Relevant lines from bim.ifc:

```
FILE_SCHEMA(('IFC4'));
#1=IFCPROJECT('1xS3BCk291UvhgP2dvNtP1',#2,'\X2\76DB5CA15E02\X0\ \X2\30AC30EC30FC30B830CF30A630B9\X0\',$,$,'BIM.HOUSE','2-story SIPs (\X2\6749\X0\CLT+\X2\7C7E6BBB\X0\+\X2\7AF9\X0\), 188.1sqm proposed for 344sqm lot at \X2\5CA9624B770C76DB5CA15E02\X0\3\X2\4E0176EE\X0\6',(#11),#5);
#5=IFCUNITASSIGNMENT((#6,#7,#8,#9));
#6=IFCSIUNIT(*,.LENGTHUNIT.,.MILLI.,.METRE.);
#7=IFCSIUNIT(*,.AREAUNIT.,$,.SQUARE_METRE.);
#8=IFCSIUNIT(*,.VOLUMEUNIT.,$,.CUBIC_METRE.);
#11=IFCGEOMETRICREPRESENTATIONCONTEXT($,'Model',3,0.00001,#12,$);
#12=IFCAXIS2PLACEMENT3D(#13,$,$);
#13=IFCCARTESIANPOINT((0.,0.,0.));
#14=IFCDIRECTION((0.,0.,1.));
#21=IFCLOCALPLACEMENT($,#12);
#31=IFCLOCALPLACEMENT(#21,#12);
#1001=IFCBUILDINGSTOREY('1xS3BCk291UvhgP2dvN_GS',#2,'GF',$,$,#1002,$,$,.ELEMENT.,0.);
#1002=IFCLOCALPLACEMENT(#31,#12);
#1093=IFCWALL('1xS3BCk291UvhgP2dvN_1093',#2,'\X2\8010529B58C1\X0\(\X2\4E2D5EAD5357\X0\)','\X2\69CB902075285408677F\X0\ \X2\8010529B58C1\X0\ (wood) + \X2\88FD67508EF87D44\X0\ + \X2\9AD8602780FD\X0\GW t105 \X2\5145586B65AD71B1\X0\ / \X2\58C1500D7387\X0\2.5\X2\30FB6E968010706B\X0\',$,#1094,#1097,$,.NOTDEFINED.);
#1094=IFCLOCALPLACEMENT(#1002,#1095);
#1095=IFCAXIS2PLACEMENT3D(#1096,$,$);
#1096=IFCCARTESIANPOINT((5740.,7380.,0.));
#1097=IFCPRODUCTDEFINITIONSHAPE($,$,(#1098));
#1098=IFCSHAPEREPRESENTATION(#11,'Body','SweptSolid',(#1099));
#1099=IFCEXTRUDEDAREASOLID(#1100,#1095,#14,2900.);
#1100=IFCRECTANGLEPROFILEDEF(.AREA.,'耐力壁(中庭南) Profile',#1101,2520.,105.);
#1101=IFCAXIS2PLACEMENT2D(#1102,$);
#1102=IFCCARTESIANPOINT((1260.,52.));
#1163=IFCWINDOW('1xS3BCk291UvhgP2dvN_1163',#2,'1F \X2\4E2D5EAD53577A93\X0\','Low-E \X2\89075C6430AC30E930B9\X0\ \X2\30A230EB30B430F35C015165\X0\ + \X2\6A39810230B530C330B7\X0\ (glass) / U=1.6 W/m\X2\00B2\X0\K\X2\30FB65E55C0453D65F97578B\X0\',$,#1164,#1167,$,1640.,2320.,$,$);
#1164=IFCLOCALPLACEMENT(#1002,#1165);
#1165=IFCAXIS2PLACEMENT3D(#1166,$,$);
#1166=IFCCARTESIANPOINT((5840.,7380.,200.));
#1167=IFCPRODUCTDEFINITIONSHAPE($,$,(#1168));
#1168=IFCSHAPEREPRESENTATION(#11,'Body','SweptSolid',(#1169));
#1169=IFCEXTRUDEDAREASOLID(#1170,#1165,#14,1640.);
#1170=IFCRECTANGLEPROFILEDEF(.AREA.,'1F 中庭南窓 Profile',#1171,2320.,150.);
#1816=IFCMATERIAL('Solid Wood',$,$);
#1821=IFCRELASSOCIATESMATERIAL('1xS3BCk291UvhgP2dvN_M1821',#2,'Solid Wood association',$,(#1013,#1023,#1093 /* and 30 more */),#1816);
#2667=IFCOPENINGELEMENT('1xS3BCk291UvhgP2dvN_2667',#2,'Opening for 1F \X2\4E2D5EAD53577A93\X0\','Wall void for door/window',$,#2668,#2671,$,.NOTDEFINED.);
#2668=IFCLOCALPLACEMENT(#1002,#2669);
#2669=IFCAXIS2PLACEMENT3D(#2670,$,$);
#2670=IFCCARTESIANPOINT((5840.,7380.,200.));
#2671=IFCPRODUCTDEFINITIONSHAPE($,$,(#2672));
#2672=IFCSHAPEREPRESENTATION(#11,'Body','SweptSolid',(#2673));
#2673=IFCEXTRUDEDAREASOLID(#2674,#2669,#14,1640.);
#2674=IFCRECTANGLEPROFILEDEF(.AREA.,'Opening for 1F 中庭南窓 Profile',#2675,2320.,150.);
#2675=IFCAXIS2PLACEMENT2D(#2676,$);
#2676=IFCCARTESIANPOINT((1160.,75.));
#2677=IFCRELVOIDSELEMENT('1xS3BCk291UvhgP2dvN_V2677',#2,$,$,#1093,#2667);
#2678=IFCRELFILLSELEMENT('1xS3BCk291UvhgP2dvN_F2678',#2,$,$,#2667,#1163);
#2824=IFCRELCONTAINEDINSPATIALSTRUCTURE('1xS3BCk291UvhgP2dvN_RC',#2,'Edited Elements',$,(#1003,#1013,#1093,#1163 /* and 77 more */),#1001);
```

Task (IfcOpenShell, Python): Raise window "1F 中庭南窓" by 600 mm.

```python
import numpy as np
import ifcopenshell
import ifcopenshell.api.geometry
import ifcopenshell.util.placement
import ifcopenshell.util.unit

model = ifcopenshell.open("bim.ifc")
unit_scale = ifcopenshell.util.unit.calculate_unit_scale(model)

window = model.by_id(1163)
opening = window.FillsVoids[0].RelatingOpeningElement
dz = 0.6 / unit_scale

shift = np.array([0.0, 0.0, dz])
# The window is not placed relative to its opening, so move both.
for product in (opening, window):
    matrix = ifcopenshell.util.placement.get_local_placement(product.ObjectPlacement)
    matrix[:3, 3] += shift
    ifcopenshell.api.geometry.edit_object_placement(model, product=product, matrix=matrix, is_si=False)

print(f"moved by {dz * unit_scale:+.3f} m")

model.write("bim_v2.ifc")
```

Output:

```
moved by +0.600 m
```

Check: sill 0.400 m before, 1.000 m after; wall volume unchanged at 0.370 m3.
